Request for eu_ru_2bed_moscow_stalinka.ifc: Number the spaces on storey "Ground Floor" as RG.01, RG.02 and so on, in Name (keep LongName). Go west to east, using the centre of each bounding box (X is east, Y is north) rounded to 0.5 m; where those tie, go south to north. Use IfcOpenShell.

First a look at what the model holds.

```python
import ifcopenshell
import ifcopenshell.util.element
import ifcopenshell.util.placement

model = ifcopenshell.open("eu_ru_2bed_moscow_stalinka.ifc")
print(model.schema)
storey = next(s for s in model.by_type("IfcBuildingStorey") if s.Name == "Ground Floor")
spaces = [e for e in ifcopenshell.util.element.get_decomposition(storey) if e.is_a("IfcSpace")]
for e in sorted(spaces, key=lambda e: e.id()):
    origin = ifcopenshell.util.placement.get_local_placement(e.ObjectPlacement)[:3, 3]
    print(e.id(), e.Name, e.LongName, origin.round(2) + 0.0, sep=" | ")
```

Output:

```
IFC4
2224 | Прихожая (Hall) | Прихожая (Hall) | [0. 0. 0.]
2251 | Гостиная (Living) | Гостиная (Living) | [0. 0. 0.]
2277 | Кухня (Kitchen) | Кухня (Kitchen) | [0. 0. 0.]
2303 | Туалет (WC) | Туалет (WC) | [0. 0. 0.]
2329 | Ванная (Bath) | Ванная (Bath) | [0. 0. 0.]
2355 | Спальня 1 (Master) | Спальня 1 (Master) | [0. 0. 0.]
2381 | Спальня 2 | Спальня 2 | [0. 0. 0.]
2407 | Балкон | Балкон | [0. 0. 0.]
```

```python
import ifcopenshell
import ifcopenshell.geom
import ifcopenshell.util.element
import ifcopenshell.util.shape

model = ifcopenshell.open("eu_ru_2bed_moscow_stalinka.ifc")
settings = ifcopenshell.geom.settings()
settings.set("use-world-coords", True)


def centre(element):
    shape = ifcopenshell.geom.create_shape(settings, element)
    return ifcopenshell.util.shape.get_bbox_centroid(shape.geometry)


storey = next(s for s in model.by_type("IfcBuildingStorey") if s.Name == "Ground Floor")
spaces = [e for e in ifcopenshell.util.element.get_decomposition(storey) if e.is_a("IfcSpace")]

# Insertion points can sit at a corner or the storey origin, so sort by the geometry (in metres).
centres = {e: centre(e) for e in spaces}
spaces.sort(key=lambda e: (round(centres[e][0] / 0.5), centres[e][1]))

for i, e in enumerate(spaces, start=1):
    number = f"RG.{i:02d}"
    e.Name = number
    print(e.id(), number)

model.write("eu_ru_2bed_moscow_stalinka_updated.ifc")
```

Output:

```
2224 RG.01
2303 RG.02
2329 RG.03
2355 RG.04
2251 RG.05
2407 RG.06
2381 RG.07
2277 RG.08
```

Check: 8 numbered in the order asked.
